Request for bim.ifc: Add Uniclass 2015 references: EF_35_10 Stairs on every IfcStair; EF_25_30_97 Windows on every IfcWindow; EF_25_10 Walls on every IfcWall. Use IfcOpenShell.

First a look at what the model holds.

```python
import ifcopenshell

model = ifcopenshell.open("bim.ifc")
print(model.schema)
print("classifications:", [c.Name for c in model.by_type("IfcClassification")])
for ifc_class in ("IfcDoor", "IfcRoof", "IfcStair", "IfcWall", "IfcWindow"):
    print(ifc_class, len(model.by_type(ifc_class)))
```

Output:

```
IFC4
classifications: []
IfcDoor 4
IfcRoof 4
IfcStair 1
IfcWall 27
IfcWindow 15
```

```python
import ifcopenshell
import ifcopenshell.api.classification

model = ifcopenshell.open("bim.ifc")

system = ifcopenshell.api.classification.add_classification(model, classification="Uniclass 2015")

codes = {
    "IfcStair": ("EF_35_10", "Stairs"),
    "IfcWindow": ("EF_25_30_97", "Windows"),
    "IfcWall": ("EF_25_10", "Walls"),
}
for ifc_class, (code, name) in codes.items():
    products = model.by_type(ifc_class)
    ifcopenshell.api.classification.add_reference(
        model, products=products, classification=system, identification=code, name=name
    )
    print(code, len(products))

model.write("bim-out.ifc")
```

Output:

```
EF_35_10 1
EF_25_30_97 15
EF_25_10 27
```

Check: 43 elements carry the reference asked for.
